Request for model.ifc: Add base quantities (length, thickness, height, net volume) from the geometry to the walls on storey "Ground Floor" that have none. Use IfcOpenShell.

First a look at what the model holds.

```python
import ifcopenshell
import ifcopenshell.util.element
import ifcopenshell.util.unit

model = ifcopenshell.open("model.ifc")
print(model.schema)
for unit_type in ("LENGTHUNIT", "AREAUNIT", "VOLUMEUNIT"):
    print(unit_type, ifcopenshell.util.unit.calculate_unit_scale(model, unit_type))
storey = next(s for s in model.by_type("IfcBuildingStorey") if s.Name == "Ground Floor")
walls = [e for e in ifcopenshell.util.element.get_decomposition(storey) if e.is_a("IfcWall")]
for e in sorted(walls, key=lambda e: e.id()):
    print(e.id(), e.is_a(), e.Name, list(ifcopenshell.util.element.get_psets(e, qtos_only=True)), sep=" | ")
```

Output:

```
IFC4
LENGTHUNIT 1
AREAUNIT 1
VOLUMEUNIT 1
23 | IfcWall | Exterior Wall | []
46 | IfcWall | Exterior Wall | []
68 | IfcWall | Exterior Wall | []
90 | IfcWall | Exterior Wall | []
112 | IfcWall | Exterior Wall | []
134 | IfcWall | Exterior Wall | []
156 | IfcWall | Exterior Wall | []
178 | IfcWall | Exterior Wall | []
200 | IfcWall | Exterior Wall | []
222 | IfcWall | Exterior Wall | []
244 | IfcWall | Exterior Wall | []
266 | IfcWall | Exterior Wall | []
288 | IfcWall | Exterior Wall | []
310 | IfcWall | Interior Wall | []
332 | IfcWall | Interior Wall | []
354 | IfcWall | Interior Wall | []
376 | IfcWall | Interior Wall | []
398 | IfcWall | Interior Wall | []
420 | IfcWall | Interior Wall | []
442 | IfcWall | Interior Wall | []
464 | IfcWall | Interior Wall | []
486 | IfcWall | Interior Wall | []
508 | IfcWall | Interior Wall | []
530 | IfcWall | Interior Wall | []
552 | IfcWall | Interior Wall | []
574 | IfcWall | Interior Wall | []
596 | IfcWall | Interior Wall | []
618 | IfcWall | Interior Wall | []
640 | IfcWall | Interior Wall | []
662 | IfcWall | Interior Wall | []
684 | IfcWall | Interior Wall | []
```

```python
import ifcopenshell
import ifcopenshell.api.pset
import ifcopenshell.geom
import ifcopenshell.util.element
import ifcopenshell.util.shape
import ifcopenshell.util.unit

model = ifcopenshell.open("model.ifc")
unit_scale = ifcopenshell.util.unit.calculate_unit_scale(model)
volume_scale = ifcopenshell.util.unit.calculate_unit_scale(model, "VOLUMEUNIT")
settings = ifcopenshell.geom.settings()

storey = next(s for s in model.by_type("IfcBuildingStorey") if s.Name == "Ground Floor")
walls = [e for e in ifcopenshell.util.element.get_decomposition(storey) if e.is_a("IfcWall")]

for e in sorted(walls, key=lambda e: e.id()):
    if ifcopenshell.util.element.get_psets(e, qtos_only=True, should_inherit=False):
        continue
    # Geometry comes back in metres, in the element's own axes.
    shape = ifcopenshell.geom.create_shape(settings, e)
    values = {
        "Length": ifcopenshell.util.shape.get_x(shape.geometry) / unit_scale,
        "Width": ifcopenshell.util.shape.get_y(shape.geometry) / unit_scale,
        "Height": ifcopenshell.util.shape.get_z(shape.geometry) / unit_scale,
        "NetVolume": ifcopenshell.util.shape.get_volume(shape.geometry) / volume_scale,
    }
    qto = ifcopenshell.api.pset.add_qto(model, product=e, name="Qto_WallBaseQuantities")
    ifcopenshell.api.pset.edit_qto(model, qto=qto, properties=values)
    print(e.id(), {k: round(v, 3) for k, v in values.items()})

model.write("model_rev.ifc")
```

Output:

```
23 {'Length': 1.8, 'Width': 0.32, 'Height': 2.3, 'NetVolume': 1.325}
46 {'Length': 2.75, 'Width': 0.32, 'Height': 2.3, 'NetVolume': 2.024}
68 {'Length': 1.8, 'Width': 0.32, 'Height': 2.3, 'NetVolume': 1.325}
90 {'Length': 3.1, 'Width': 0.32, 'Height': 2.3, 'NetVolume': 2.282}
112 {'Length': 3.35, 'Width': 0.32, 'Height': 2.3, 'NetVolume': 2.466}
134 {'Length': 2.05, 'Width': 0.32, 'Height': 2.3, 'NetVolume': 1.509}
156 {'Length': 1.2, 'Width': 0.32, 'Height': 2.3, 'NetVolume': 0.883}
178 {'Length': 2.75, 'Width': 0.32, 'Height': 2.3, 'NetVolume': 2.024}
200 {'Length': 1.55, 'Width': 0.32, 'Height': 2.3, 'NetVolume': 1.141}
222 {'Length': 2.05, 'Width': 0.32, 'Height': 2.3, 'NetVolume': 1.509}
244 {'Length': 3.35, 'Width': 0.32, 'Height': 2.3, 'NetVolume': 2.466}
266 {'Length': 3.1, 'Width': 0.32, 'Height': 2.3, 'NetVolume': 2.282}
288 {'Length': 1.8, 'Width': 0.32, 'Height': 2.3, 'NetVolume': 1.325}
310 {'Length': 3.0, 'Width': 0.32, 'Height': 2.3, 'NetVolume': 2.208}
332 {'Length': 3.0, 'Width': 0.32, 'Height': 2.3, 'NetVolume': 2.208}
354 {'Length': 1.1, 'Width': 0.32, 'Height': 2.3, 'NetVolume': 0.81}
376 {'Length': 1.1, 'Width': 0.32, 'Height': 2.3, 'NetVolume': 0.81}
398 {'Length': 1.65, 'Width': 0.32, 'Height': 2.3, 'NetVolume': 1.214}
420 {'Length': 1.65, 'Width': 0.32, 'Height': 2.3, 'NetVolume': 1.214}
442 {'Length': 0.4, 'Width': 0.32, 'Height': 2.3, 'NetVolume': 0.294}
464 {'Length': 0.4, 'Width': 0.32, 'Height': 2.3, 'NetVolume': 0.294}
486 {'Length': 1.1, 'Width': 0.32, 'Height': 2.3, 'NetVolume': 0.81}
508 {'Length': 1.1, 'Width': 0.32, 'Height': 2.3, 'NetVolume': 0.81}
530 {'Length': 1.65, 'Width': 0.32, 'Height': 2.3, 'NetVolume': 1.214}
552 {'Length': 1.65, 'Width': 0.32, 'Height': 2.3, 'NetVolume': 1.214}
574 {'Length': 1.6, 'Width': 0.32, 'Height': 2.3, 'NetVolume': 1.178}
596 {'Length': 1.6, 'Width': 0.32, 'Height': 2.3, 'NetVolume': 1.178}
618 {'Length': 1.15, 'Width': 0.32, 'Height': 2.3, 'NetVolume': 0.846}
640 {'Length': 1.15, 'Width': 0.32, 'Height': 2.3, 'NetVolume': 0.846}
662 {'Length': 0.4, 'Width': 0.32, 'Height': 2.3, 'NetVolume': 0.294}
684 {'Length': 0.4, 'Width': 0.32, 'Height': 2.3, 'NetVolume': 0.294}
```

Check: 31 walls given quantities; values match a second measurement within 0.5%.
